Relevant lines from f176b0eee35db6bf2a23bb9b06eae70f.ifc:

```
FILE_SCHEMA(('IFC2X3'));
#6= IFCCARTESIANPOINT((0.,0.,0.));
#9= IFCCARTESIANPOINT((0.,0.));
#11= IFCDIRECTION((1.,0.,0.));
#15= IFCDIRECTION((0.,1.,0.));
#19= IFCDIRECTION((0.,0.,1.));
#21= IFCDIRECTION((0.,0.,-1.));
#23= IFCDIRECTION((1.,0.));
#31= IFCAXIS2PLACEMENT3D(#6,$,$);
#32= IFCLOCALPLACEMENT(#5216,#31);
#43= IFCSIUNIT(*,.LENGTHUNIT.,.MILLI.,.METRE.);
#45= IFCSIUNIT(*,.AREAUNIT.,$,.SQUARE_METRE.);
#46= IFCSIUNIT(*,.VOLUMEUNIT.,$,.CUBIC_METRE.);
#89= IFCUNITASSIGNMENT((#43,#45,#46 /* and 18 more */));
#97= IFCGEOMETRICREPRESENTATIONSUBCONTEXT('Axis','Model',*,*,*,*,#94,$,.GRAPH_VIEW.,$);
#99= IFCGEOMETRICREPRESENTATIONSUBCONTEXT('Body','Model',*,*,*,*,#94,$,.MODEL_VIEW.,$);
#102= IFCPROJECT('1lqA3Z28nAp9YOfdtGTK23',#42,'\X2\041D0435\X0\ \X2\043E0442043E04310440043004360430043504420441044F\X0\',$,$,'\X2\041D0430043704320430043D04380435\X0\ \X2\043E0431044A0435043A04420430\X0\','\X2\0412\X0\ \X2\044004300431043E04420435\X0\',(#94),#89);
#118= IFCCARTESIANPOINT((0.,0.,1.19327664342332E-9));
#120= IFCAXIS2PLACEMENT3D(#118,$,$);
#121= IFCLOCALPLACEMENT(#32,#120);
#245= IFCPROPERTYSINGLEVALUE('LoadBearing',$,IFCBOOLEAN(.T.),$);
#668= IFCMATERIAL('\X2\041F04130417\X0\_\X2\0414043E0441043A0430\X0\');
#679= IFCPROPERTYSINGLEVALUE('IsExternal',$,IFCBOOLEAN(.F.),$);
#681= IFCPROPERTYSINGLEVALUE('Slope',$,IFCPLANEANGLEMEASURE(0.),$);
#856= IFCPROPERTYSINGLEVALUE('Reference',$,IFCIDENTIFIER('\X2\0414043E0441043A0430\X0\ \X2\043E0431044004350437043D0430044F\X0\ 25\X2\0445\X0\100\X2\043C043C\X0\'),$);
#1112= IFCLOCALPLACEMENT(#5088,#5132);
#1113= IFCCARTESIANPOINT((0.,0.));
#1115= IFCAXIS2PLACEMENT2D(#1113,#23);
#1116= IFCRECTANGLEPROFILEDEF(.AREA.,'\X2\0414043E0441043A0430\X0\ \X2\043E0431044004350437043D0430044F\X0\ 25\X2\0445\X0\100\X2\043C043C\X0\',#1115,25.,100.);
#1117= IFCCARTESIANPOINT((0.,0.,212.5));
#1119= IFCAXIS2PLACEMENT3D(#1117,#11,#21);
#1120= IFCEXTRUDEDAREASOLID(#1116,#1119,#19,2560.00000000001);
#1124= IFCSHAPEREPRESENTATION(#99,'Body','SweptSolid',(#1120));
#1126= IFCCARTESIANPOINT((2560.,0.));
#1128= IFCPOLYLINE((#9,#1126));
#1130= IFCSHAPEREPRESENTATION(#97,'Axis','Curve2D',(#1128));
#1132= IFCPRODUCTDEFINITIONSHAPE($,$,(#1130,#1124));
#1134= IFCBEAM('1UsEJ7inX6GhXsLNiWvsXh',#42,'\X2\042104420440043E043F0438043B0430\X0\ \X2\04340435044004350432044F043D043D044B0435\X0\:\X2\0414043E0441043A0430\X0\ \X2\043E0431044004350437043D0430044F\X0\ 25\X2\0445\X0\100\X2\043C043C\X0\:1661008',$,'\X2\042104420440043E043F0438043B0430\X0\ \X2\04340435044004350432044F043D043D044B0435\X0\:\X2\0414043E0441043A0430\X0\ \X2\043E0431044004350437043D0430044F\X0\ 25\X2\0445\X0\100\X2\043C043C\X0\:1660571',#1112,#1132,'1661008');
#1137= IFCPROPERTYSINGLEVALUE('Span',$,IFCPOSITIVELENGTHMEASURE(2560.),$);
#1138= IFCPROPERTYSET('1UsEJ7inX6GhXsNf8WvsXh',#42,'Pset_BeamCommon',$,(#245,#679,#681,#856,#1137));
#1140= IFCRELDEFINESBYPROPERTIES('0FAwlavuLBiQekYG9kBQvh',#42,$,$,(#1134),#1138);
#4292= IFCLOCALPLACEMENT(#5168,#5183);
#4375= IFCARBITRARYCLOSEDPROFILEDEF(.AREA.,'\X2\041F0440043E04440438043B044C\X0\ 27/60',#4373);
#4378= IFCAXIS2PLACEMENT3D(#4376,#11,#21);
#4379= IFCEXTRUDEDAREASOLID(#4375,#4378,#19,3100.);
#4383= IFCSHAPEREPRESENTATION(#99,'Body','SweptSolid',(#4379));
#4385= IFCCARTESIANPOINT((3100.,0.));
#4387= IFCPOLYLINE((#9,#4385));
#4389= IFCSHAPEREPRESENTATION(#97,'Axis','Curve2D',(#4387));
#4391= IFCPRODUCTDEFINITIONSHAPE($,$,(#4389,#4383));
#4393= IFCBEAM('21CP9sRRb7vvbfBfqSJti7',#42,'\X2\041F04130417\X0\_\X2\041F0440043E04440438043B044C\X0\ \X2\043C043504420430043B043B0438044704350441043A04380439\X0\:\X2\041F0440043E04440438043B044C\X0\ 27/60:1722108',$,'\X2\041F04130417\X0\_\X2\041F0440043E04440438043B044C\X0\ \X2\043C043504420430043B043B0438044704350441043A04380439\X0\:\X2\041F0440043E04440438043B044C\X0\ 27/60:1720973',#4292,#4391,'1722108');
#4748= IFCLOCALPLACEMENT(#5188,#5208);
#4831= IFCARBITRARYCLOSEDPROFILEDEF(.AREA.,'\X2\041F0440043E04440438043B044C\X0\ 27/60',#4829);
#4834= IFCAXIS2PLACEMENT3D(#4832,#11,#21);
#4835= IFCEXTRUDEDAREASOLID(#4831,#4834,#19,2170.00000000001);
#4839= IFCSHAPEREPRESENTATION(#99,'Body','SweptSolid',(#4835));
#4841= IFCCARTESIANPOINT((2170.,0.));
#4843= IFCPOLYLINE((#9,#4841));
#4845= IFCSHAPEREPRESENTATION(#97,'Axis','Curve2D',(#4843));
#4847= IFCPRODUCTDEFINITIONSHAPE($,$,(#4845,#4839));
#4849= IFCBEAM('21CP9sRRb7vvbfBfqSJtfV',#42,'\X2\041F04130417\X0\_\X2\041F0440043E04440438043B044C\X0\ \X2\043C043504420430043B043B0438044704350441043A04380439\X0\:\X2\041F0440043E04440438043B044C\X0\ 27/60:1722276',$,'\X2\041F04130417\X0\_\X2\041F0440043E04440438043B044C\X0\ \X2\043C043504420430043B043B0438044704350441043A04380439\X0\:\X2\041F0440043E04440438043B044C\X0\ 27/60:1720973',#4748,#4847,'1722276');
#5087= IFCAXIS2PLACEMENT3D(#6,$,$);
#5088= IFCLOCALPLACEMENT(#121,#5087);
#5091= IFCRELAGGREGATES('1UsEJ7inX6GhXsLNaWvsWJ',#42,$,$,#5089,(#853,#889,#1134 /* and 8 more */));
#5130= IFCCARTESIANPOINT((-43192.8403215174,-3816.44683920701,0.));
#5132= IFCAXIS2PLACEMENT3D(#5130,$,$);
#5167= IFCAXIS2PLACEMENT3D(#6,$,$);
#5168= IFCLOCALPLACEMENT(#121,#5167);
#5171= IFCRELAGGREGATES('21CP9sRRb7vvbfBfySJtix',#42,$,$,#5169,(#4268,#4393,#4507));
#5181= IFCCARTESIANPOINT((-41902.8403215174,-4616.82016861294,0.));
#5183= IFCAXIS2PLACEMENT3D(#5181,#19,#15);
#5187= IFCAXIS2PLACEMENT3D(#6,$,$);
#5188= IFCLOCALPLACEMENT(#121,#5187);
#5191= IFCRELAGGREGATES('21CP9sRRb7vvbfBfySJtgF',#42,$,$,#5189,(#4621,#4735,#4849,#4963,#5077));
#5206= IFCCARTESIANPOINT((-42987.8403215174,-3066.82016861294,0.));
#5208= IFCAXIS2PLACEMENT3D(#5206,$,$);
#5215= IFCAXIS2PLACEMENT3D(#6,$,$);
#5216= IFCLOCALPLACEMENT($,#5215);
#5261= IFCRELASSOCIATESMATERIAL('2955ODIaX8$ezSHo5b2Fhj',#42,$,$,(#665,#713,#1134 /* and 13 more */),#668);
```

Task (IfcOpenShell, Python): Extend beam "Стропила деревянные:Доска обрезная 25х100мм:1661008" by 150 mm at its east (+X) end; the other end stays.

```python
import numpy as np
import ifcopenshell
import ifcopenshell.api.pset
import ifcopenshell.util.element
import ifcopenshell.util.representation
import ifcopenshell.util.unit

model = ifcopenshell.open("f176b0eee35db6bf2a23bb9b06eae70f.ifc")
unit_scale = ifcopenshell.util.unit.calculate_unit_scale(model)

member = model.by_guid("1UsEJ7inX6GhXsLNiWvsXh")
change = 0.15 / unit_scale

# The extrusion runs towards the end named, so only its depth changes.
body = ifcopenshell.util.representation.get_representation(member, "Model", "Body")
solid = body.Items[0]
old_length = solid.Depth
solid.Depth += change

# Move the axis end point with it.
axis = next(r for r in member.Representation.Representations if r.RepresentationIdentifier == "Axis").Items[0]
start, end = (np.array(p.Coordinates) for p in axis.Points)
end = end + (end - start) / np.linalg.norm(end - start) * change
point = model.createIfcCartesianPoint(end.tolist())
axis.Points = [axis.Points[0], point]

# Update the stored length and volume.
pset = model.by_id(ifcopenshell.util.element.get_pset(member, "Pset_BeamCommon", should_inherit=False)["id"])
ifcopenshell.api.pset.edit_pset(model, pset=pset, properties={
    "Span": model.create_entity("IfcPositiveLengthMeasure", solid.Depth),
})

print(f"length {old_length:g} -> {solid.Depth:g}")

model.write("f176b0eee35db6bf2a23bb9b06eae70f_rev.ifc")
```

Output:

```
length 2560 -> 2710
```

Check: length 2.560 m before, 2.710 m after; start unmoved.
